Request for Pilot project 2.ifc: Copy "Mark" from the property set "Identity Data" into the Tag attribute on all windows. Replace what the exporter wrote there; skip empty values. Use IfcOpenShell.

First a look at what the model holds.

```python
import ifcopenshell
import ifcopenshell.util.element

model = ifcopenshell.open("Pilot project 2.ifc")
print(model.schema)
windows = model.by_type("IfcWindow")
print(len(windows), "windows")
for e in windows[:8]:
    source = ifcopenshell.util.element.get_pset(e, "Identity Data", "Mark")
    target = e.Tag
    print(e.id(), repr(source), repr(target), sep=" | ")
```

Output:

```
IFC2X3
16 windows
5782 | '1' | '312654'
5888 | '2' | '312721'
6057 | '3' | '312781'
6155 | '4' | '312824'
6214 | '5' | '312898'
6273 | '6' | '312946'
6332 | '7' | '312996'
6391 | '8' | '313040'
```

```python
import ifcopenshell
import ifcopenshell.util.element

model = ifcopenshell.open("Pilot project 2.ifc")

count = 0
for e in model.by_type("IfcWindow"):
    value = ifcopenshell.util.element.get_pset(e, "Identity Data", "Mark")
    current = e.Tag
    if not value or not value.strip() or current == value:
        continue
    e.Tag = value
    count += 1

print(count, "windows updated")

model.write("Pilot project 2_v2.ifc")
```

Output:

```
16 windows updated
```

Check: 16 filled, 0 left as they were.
